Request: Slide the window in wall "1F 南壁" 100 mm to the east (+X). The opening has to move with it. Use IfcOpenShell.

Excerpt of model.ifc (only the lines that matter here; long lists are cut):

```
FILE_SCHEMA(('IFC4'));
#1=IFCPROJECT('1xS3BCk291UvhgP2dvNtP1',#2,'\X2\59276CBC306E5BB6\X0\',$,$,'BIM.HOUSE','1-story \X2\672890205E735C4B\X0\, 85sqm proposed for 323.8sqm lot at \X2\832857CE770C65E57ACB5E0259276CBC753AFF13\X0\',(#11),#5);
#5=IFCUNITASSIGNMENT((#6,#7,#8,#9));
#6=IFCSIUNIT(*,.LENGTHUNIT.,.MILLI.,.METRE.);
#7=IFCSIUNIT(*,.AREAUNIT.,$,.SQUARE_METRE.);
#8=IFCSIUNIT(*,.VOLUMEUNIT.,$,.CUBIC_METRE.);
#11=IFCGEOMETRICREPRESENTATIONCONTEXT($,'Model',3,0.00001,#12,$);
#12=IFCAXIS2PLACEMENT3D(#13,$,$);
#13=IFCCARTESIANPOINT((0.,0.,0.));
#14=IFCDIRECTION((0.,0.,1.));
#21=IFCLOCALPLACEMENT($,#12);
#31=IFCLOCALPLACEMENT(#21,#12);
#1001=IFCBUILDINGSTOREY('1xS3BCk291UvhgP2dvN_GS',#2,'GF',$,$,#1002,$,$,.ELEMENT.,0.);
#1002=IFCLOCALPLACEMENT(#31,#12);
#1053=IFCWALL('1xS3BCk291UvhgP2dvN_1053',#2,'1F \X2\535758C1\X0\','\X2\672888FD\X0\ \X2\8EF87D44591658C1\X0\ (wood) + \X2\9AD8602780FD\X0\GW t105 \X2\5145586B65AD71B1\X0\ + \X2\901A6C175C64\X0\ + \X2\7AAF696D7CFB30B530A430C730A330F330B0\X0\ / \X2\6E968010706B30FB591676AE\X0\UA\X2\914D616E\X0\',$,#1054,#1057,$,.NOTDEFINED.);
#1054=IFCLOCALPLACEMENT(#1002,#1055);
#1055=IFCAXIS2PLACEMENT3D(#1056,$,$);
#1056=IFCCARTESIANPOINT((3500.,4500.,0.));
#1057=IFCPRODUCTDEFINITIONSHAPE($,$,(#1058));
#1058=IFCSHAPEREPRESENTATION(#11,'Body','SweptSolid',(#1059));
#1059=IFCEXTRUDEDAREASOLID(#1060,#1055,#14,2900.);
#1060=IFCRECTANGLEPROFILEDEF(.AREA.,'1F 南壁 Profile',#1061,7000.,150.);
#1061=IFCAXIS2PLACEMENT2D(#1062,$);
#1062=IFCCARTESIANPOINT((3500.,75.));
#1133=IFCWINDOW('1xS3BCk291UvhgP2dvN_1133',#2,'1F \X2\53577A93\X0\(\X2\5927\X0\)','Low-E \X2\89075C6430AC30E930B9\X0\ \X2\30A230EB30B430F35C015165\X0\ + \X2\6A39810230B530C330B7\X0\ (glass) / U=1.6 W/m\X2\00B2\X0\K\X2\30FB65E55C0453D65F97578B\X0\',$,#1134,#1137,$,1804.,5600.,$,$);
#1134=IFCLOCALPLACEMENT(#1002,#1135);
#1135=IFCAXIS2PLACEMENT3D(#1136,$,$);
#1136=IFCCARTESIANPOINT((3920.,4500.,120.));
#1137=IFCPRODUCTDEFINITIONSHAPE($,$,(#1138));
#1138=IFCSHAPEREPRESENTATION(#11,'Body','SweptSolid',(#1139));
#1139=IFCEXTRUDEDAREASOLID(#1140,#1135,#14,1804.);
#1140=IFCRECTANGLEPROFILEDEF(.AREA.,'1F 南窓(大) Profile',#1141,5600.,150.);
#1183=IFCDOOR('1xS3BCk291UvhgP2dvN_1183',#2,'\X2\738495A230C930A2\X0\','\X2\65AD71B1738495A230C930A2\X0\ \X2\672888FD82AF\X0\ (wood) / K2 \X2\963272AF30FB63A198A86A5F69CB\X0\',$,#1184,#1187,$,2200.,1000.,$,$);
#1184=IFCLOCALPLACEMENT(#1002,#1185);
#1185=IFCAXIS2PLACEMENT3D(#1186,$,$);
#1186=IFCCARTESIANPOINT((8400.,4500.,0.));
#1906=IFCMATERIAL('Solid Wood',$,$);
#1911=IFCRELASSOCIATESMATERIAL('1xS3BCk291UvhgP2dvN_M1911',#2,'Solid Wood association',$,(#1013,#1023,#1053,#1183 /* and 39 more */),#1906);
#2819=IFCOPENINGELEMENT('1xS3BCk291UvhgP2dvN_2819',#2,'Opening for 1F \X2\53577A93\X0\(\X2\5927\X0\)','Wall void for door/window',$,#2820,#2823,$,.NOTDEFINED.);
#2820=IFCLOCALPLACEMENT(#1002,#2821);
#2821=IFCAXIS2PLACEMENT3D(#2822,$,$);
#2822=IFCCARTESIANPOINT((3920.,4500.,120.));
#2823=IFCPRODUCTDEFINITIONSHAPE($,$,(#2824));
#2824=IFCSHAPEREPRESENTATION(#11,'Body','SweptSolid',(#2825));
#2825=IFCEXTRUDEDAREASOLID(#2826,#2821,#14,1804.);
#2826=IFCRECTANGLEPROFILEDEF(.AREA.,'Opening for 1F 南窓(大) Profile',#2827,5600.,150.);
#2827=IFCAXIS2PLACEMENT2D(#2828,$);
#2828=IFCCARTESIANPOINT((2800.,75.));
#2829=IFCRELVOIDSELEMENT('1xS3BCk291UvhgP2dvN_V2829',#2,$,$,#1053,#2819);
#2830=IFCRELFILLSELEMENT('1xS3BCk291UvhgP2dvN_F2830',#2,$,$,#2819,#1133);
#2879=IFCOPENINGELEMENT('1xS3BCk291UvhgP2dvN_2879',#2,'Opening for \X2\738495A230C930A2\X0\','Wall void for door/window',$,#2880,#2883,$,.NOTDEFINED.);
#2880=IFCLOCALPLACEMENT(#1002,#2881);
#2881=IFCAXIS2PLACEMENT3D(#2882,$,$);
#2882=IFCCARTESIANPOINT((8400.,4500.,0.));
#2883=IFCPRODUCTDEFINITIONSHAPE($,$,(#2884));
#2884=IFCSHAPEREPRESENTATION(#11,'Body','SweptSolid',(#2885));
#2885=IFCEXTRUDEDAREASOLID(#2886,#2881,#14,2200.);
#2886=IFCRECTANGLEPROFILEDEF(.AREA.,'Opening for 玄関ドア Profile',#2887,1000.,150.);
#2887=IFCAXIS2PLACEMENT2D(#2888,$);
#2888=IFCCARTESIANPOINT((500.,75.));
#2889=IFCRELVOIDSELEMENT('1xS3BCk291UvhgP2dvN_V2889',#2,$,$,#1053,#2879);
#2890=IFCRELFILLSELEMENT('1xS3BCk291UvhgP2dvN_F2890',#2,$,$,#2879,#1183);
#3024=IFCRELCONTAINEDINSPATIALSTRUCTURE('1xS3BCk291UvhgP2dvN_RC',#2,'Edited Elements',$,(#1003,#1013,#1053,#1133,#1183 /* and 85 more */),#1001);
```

```python
import ifcopenshell
import ifcopenshell.api.geometry
import ifcopenshell.util.placement
import ifcopenshell.util.unit

model = ifcopenshell.open("model.ifc")
unit_scale = ifcopenshell.util.unit.calculate_unit_scale(model)

window = model.by_id(1133)
opening = window.FillsVoids[0].RelatingOpeningElement
wall = opening.VoidsElements[0].RelatingBuildingElement

wall_matrix = ifcopenshell.util.placement.get_local_placement(wall.ObjectPlacement)
shift = wall_matrix[:3, 0] * 0.1 / unit_scale
before = ifcopenshell.util.placement.get_local_placement(window.ObjectPlacement)[:3, 3].copy()

# The window is not placed relative to its opening, so move both.
for product in (opening, window):
    matrix = ifcopenshell.util.placement.get_local_placement(product.ObjectPlacement)
    matrix[:3, 3] += shift
    ifcopenshell.api.geometry.edit_object_placement(model, product=product, matrix=matrix, is_si=False)

after = ifcopenshell.util.placement.get_local_placement(window.ObjectPlacement)[:3, 3]
print("window moved by", (after - before).round(3) + 0.0)

model.write("model_edited.ifc")
```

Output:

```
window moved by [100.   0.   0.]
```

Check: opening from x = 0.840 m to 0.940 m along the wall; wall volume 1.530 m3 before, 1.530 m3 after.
